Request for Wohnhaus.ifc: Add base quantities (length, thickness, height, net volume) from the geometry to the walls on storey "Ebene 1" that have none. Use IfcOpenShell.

First a look at what the model holds.

```python
import ifcopenshell
import ifcopenshell.util.element
import ifcopenshell.util.unit

model = ifcopenshell.open("Wohnhaus.ifc")
print(model.schema)
for unit_type in ("LENGTHUNIT", "AREAUNIT", "VOLUMEUNIT"):
    print(unit_type, ifcopenshell.util.unit.calculate_unit_scale(model, unit_type))
storey = next(s for s in model.by_type("IfcBuildingStorey") if s.Name == "Ebene 1")
walls = [e for e in ifcopenshell.util.element.get_decomposition(storey) if e.is_a("IfcWall")]
for e in sorted(walls, key=lambda e: e.id()):
    print(e.id(), e.is_a(), e.Name, list(ifcopenshell.util.element.get_psets(e, qtos_only=True)), sep=" | ")
```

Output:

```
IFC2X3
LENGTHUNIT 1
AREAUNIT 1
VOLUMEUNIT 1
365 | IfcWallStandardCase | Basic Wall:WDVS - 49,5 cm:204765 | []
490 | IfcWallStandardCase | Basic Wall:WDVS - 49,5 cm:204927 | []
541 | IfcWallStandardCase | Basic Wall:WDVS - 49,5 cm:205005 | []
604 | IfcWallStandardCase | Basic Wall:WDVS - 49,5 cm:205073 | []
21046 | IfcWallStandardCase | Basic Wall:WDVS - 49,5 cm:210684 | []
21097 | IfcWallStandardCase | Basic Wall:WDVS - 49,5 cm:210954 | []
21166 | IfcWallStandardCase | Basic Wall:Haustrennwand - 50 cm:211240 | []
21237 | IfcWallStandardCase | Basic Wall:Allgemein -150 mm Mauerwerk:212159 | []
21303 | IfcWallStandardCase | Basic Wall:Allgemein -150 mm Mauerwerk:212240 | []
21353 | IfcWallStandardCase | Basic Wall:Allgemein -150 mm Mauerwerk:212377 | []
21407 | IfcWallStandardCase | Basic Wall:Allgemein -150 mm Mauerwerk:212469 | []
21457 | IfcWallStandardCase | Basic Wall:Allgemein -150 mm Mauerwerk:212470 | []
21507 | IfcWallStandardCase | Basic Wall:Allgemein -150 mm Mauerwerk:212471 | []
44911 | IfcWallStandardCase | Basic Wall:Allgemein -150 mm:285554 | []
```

```python
import ifcopenshell
import ifcopenshell.api.pset
import ifcopenshell.geom
import ifcopenshell.util.element
import ifcopenshell.util.shape
import ifcopenshell.util.unit

model = ifcopenshell.open("Wohnhaus.ifc")
unit_scale = ifcopenshell.util.unit.calculate_unit_scale(model)
volume_scale = ifcopenshell.util.unit.calculate_unit_scale(model, "VOLUMEUNIT")
settings = ifcopenshell.geom.settings()

storey = next(s for s in model.by_type("IfcBuildingStorey") if s.Name == "Ebene 1")
walls = [e for e in ifcopenshell.util.element.get_decomposition(storey) if e.is_a("IfcWall")]

for e in sorted(walls, key=lambda e: e.id()):
    if ifcopenshell.util.element.get_psets(e, qtos_only=True, should_inherit=False):
        continue
    # Geometry comes back in metres, in the element's own axes.
    shape = ifcopenshell.geom.create_shape(settings, e)
    values = {
        "Length": ifcopenshell.util.shape.get_x(shape.geometry) / unit_scale,
        "Width": ifcopenshell.util.shape.get_y(shape.geometry) / unit_scale,
        "Height": ifcopenshell.util.shape.get_z(shape.geometry) / unit_scale,
        "NetVolume": ifcopenshell.util.shape.get_volume(shape.geometry) / volume_scale,
    }
    qto = ifcopenshell.api.pset.add_qto(model, product=e, name="BaseQuantities")
    ifcopenshell.api.pset.edit_qto(model, qto=qto, properties=values)
    print(e.id(), {k: round(v, 3) for k, v in values.items()})

model.write("Wohnhaus-out.ifc")
```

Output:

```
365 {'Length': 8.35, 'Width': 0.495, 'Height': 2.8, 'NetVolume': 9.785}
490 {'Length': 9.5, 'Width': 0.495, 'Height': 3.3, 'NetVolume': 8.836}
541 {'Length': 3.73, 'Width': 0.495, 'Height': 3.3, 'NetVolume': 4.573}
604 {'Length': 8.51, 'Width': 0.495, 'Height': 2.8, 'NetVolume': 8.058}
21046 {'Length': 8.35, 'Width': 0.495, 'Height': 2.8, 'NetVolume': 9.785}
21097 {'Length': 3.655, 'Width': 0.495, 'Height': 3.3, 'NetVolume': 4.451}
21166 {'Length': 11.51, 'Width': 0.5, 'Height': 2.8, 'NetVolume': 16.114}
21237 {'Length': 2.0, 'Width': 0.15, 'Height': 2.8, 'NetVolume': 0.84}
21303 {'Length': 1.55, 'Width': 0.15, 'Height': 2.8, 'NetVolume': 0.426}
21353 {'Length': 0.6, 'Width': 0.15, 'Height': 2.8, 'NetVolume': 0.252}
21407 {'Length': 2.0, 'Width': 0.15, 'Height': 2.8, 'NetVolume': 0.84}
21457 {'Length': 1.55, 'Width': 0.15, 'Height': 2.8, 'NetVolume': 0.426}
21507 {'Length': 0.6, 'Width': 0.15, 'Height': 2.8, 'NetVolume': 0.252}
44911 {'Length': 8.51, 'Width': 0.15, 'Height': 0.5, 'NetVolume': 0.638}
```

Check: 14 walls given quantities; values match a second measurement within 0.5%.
